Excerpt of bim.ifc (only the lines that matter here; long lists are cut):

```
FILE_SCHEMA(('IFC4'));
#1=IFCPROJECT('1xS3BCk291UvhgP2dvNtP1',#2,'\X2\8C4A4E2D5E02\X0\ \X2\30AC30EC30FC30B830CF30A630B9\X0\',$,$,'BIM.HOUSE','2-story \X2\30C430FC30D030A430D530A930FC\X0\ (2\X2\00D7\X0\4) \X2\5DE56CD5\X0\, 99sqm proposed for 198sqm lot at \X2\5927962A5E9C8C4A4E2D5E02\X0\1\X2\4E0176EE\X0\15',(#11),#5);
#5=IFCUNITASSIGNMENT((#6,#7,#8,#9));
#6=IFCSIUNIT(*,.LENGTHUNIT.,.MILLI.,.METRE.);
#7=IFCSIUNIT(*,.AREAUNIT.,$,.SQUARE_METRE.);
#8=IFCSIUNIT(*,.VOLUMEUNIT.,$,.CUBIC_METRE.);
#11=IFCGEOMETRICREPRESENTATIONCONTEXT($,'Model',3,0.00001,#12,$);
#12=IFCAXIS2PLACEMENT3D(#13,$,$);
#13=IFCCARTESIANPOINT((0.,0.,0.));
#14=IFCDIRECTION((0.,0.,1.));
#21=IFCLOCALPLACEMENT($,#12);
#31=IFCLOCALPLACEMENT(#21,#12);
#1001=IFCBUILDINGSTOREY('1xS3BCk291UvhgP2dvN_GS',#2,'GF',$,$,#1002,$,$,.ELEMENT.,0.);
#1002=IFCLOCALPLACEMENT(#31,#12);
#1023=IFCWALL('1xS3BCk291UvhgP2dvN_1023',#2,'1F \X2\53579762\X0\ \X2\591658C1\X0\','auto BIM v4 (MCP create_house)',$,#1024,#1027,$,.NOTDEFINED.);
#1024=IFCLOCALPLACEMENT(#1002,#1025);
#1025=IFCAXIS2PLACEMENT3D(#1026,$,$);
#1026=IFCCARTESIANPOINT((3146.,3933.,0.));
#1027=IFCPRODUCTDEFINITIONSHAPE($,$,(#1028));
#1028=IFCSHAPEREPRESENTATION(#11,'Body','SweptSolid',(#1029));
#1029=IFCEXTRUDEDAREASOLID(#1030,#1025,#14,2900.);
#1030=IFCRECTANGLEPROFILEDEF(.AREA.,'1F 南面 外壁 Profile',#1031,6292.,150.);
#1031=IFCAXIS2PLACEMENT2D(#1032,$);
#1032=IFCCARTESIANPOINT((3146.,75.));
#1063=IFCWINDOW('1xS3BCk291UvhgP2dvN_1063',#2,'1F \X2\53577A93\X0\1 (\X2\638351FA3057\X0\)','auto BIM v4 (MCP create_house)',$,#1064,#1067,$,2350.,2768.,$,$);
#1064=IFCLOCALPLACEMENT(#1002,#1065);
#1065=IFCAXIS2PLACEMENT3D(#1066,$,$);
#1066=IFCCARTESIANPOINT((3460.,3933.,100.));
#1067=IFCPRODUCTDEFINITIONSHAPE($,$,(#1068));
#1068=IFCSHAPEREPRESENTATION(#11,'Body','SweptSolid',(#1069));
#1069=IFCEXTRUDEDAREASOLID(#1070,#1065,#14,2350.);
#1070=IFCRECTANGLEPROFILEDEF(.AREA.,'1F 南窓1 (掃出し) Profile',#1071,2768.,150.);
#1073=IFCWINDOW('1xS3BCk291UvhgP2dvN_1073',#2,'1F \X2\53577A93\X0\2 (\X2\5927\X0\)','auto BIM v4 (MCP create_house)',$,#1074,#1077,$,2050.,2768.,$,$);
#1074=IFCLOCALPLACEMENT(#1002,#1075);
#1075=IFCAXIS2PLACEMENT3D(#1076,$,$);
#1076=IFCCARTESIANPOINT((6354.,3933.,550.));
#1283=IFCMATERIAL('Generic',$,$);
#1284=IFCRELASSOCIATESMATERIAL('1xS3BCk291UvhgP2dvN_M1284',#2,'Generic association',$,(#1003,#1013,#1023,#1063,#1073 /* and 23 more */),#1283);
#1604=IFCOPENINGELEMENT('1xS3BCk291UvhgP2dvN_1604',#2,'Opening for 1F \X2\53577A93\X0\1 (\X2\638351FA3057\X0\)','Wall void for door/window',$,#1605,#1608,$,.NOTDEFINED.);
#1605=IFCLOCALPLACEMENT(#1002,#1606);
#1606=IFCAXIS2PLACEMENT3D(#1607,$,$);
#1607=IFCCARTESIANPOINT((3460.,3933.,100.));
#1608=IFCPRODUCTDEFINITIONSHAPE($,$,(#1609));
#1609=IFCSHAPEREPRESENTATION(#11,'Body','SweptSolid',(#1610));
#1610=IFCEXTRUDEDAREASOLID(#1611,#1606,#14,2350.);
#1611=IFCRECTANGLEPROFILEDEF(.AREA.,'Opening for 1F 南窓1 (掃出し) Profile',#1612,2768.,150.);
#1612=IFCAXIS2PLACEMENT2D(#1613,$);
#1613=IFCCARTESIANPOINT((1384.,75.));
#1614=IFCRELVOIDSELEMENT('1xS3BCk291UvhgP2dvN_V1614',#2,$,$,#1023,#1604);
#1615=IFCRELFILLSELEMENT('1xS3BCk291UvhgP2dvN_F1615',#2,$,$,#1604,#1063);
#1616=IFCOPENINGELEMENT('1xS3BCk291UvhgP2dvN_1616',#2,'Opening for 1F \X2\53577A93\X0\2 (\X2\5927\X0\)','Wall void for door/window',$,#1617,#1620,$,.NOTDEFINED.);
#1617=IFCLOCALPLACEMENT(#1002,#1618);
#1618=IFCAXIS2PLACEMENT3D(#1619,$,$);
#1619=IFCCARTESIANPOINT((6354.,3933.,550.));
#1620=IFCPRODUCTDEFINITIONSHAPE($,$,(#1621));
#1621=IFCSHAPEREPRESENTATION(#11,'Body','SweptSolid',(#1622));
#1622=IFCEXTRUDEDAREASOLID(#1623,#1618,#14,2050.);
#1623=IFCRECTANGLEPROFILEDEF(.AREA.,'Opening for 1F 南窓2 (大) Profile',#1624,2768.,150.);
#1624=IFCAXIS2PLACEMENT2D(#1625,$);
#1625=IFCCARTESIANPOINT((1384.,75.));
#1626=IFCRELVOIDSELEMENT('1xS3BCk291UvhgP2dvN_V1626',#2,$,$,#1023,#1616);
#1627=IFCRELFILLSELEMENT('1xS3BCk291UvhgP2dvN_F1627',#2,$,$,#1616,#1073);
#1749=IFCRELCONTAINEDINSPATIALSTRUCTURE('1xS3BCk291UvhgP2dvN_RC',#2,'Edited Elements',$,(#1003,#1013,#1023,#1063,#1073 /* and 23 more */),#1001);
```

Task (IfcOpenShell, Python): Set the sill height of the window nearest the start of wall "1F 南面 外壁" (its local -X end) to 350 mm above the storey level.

```python
import numpy as np
import ifcopenshell
import ifcopenshell.api.geometry
import ifcopenshell.geom
import ifcopenshell.util.element
import ifcopenshell.util.placement
import ifcopenshell.util.shape
import ifcopenshell.util.unit

model = ifcopenshell.open("bim.ifc")
unit_scale = ifcopenshell.util.unit.calculate_unit_scale(model)

window = model.by_guid("1xS3BCk291UvhgP2dvN_1063")
opening = window.FillsVoids[0].RelatingOpeningElement
storey = ifcopenshell.util.element.get_container(window, ifc_class="IfcBuildingStorey")
level = ifcopenshell.util.placement.get_local_placement(storey.ObjectPlacement)[2, 3]

# The opening's origin need not be at the sill, so measure its lowest point.
shape = ifcopenshell.geom.create_shape(ifcopenshell.geom.settings(), opening)
bottom = ifcopenshell.util.shape.get_shape_bottom_elevation(shape, shape.geometry) / unit_scale
dz = level + 0.35 / unit_scale - bottom

shift = np.array([0.0, 0.0, dz])
# The window is not placed relative to its opening, so move both.
for product in (opening, window):
    matrix = ifcopenshell.util.placement.get_local_placement(product.ObjectPlacement)
    matrix[:3, 3] += shift
    ifcopenshell.api.geometry.edit_object_placement(model, product=product, matrix=matrix, is_si=False)

print(f"moved by {dz * unit_scale:+.3f} m")

model.write("bim_edited.ifc")
```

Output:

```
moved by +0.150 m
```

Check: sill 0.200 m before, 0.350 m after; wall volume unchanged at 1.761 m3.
